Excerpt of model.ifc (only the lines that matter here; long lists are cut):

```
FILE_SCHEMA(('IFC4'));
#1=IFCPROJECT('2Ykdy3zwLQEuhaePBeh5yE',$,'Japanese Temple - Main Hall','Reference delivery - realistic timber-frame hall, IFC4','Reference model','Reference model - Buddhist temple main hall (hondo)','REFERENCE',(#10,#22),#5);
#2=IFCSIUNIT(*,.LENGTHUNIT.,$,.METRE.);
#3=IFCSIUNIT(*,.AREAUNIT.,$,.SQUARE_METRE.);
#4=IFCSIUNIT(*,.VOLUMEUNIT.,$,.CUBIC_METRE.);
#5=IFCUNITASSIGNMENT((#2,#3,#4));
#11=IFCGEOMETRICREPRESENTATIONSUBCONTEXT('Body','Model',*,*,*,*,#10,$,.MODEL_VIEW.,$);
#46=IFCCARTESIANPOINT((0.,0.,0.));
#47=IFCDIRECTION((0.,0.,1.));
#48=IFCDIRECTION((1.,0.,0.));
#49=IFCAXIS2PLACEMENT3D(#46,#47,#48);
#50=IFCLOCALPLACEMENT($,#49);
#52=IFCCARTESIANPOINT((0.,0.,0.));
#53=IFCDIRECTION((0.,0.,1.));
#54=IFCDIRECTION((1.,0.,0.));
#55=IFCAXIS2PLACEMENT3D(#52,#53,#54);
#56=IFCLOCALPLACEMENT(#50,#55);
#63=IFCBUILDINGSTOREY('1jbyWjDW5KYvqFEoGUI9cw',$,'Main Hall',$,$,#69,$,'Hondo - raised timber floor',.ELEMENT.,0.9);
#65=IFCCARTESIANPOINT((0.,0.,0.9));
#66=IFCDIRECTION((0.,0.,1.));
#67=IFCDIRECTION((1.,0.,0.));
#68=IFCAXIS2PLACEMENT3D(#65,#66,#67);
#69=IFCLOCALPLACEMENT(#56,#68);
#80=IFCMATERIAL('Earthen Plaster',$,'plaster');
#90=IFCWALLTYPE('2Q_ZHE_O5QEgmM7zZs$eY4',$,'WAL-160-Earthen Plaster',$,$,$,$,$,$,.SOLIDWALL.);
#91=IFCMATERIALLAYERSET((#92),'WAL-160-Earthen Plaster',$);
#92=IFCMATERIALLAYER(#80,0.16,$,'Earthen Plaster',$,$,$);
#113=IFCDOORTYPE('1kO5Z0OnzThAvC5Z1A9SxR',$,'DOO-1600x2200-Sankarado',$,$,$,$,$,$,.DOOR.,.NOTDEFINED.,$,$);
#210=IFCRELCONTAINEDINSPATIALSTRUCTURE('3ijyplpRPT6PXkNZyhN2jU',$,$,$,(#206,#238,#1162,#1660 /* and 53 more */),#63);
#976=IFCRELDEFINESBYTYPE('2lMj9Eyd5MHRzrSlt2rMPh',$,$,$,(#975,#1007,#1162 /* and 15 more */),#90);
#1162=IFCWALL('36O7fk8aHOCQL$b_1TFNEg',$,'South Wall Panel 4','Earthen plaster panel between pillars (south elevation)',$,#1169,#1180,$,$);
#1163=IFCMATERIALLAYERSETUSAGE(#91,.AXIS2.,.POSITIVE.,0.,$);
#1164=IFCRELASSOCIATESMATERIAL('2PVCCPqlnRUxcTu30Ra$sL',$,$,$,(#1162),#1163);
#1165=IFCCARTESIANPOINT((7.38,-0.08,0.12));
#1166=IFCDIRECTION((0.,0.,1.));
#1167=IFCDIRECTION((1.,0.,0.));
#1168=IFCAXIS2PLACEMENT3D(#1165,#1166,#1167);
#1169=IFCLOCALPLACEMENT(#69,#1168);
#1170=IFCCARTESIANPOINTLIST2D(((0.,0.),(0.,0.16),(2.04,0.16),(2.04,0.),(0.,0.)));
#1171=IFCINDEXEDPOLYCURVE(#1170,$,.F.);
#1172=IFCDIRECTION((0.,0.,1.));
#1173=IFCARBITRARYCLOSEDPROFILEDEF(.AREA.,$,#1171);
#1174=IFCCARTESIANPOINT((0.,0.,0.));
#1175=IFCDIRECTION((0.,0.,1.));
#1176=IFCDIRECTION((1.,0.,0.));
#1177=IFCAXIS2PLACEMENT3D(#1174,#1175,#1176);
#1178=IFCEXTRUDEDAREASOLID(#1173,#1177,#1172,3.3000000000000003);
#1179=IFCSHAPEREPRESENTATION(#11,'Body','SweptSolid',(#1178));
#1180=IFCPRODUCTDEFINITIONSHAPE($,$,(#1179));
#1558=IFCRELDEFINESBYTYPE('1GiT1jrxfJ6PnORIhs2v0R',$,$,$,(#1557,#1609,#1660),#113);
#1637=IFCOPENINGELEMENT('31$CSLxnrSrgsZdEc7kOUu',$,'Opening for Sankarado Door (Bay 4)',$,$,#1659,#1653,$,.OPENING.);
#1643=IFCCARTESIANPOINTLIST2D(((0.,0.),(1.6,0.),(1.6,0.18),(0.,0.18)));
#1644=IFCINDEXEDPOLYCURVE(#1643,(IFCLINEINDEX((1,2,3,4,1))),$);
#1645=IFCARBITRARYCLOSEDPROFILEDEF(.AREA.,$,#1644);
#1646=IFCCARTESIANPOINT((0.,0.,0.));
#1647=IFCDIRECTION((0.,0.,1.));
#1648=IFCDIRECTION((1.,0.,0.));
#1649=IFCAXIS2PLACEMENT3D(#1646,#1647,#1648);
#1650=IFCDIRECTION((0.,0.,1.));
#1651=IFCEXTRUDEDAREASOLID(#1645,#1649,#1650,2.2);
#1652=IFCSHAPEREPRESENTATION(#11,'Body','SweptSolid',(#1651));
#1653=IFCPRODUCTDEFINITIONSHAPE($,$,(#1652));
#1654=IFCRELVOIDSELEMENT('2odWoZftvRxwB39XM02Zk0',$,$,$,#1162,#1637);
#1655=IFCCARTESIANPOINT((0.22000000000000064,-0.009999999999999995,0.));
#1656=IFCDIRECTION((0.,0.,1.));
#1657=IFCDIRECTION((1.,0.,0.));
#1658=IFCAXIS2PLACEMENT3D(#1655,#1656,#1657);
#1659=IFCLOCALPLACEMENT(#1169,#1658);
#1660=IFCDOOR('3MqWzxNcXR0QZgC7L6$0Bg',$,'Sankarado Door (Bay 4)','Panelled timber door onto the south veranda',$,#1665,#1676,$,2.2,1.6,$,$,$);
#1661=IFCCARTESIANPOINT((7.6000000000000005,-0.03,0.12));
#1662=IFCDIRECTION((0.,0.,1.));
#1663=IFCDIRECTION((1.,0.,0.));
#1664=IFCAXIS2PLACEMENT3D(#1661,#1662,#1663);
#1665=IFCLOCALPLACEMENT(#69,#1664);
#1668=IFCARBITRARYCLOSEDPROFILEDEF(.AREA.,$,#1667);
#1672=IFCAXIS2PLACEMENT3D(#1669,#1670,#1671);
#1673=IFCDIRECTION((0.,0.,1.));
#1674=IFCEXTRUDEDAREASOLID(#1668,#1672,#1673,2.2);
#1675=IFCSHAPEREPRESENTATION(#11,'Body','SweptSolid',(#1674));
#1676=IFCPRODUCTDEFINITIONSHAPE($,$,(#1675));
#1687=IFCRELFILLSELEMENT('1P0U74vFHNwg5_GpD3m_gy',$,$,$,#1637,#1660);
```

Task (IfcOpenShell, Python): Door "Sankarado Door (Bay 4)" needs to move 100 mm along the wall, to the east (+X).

```python
import ifcopenshell
import ifcopenshell.api.geometry
import ifcopenshell.util.placement
import ifcopenshell.util.unit

model = ifcopenshell.open("model.ifc")
unit_scale = ifcopenshell.util.unit.calculate_unit_scale(model)

door = model.by_id(1660)
opening = door.FillsVoids[0].RelatingOpeningElement
wall = opening.VoidsElements[0].RelatingBuildingElement

wall_matrix = ifcopenshell.util.placement.get_local_placement(wall.ObjectPlacement)
shift = wall_matrix[:3, 0] * 0.1 / unit_scale
before = ifcopenshell.util.placement.get_local_placement(door.ObjectPlacement)[:3, 3].copy()

# The door is not placed relative to its opening, so move both.
for product in (opening, door):
    matrix = ifcopenshell.util.placement.get_local_placement(product.ObjectPlacement)
    matrix[:3, 3] += shift
    ifcopenshell.api.geometry.edit_object_placement(model, product=product, matrix=matrix, is_si=False)

after = ifcopenshell.util.placement.get_local_placement(door.ObjectPlacement)[:3, 3]
print("door moved by", (after - before).round(3) + 0.0)

model.write("model_rev.ifc")
```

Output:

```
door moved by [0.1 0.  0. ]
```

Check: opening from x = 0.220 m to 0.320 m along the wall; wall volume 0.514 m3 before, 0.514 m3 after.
